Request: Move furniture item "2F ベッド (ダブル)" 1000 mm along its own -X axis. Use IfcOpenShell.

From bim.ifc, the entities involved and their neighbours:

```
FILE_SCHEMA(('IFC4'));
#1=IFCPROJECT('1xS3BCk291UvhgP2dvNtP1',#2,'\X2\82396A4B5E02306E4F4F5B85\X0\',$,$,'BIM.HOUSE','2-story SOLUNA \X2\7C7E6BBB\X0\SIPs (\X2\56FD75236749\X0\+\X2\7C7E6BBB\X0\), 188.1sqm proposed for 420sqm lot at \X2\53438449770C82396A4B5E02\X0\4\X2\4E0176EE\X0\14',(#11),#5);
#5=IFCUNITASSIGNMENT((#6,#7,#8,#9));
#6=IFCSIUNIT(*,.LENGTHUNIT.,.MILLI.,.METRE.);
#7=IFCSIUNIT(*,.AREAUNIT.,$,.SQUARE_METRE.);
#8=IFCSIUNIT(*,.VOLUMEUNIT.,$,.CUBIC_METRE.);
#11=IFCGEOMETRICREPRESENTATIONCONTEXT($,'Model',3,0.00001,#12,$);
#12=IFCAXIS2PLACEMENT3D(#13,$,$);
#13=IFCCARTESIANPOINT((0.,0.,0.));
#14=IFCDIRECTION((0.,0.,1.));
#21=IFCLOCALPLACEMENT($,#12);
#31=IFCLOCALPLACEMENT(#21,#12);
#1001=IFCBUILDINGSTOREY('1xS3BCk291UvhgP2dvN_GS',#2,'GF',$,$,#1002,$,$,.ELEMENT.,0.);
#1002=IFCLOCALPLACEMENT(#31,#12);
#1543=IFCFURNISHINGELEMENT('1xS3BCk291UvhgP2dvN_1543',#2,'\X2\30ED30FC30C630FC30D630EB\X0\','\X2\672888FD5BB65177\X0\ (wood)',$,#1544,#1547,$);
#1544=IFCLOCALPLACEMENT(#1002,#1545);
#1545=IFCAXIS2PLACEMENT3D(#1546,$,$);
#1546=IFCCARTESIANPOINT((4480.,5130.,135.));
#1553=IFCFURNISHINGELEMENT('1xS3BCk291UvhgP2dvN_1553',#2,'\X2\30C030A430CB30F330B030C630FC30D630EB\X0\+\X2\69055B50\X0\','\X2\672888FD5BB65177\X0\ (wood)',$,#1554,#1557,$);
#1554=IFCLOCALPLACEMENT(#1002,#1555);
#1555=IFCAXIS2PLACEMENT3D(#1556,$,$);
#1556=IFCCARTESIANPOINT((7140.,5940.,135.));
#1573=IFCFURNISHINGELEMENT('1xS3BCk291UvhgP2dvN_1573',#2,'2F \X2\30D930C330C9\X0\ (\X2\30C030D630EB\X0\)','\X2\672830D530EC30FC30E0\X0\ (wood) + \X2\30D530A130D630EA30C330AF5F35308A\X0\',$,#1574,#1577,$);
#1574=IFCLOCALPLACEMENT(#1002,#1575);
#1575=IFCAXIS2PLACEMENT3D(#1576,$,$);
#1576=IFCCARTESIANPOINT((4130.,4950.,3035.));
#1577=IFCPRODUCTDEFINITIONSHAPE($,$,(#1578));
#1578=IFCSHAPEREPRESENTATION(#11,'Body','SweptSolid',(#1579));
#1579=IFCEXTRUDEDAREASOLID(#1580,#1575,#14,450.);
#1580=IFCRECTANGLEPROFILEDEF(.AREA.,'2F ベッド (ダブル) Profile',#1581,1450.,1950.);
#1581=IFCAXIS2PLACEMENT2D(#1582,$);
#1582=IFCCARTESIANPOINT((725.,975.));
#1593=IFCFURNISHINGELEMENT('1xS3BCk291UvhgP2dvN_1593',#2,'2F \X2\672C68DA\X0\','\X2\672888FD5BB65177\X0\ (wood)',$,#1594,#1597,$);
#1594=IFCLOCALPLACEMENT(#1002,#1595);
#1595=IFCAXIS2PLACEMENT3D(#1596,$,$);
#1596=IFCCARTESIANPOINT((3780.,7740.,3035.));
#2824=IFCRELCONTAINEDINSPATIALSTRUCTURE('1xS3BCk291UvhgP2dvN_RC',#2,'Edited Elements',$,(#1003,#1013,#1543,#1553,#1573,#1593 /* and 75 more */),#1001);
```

```python
import ifcopenshell
import ifcopenshell.api.geometry
import ifcopenshell.util.placement
import ifcopenshell.util.unit

model = ifcopenshell.open("bim.ifc")
unit_scale = ifcopenshell.util.unit.calculate_unit_scale(model)

item = model.by_id(1573)
matrix = ifcopenshell.util.placement.get_local_placement(item.ObjectPlacement)
matrix[:3, 3] -= matrix[:3, 0] * 1 / unit_scale
ifcopenshell.api.geometry.edit_object_placement(model, product=item, matrix=matrix, is_si=False)

print(ifcopenshell.util.placement.get_local_placement(item.ObjectPlacement).round(3) + 0.0)

model.write("bim_v2.ifc")
```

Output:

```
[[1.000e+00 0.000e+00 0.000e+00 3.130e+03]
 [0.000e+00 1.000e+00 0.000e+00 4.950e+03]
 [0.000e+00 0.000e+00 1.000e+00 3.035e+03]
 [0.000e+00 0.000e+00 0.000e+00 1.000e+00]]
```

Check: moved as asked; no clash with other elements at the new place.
